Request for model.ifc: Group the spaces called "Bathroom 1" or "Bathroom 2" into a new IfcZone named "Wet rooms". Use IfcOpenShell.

First a look at what the model holds.

```python
import ifcopenshell

model = ifcopenshell.open("model.ifc")
print(model.schema)
seen = {}
for space in model.by_type("IfcSpace"):
    seen[space.LongName] = seen.get(space.LongName, 0) + 1
for name, count in sorted(seen.items(), key=str):
    print(count, "x", name)
print("zones:", [z.Name for z in model.by_type("IfcZone")][:20])
```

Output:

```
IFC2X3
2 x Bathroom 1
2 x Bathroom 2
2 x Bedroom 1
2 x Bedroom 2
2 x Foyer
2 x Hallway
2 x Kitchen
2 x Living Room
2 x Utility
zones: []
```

```python
import ifcopenshell
import ifcopenshell.api.group
import ifcopenshell.api.root

model = ifcopenshell.open("model.ifc")

names = {"Bathroom 1", "Bathroom 2"}
spaces = [s for s in model.by_type("IfcSpace") if s.LongName in names]

zone = ifcopenshell.api.root.create_entity(model, ifc_class="IfcZone", name="Wet rooms")
ifcopenshell.api.group.assign_group(model, products=spaces, group=zone)
print(len(spaces), "spaces in", zone.Name)

model.write("model-out.ifc")
```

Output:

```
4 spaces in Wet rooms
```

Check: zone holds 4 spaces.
